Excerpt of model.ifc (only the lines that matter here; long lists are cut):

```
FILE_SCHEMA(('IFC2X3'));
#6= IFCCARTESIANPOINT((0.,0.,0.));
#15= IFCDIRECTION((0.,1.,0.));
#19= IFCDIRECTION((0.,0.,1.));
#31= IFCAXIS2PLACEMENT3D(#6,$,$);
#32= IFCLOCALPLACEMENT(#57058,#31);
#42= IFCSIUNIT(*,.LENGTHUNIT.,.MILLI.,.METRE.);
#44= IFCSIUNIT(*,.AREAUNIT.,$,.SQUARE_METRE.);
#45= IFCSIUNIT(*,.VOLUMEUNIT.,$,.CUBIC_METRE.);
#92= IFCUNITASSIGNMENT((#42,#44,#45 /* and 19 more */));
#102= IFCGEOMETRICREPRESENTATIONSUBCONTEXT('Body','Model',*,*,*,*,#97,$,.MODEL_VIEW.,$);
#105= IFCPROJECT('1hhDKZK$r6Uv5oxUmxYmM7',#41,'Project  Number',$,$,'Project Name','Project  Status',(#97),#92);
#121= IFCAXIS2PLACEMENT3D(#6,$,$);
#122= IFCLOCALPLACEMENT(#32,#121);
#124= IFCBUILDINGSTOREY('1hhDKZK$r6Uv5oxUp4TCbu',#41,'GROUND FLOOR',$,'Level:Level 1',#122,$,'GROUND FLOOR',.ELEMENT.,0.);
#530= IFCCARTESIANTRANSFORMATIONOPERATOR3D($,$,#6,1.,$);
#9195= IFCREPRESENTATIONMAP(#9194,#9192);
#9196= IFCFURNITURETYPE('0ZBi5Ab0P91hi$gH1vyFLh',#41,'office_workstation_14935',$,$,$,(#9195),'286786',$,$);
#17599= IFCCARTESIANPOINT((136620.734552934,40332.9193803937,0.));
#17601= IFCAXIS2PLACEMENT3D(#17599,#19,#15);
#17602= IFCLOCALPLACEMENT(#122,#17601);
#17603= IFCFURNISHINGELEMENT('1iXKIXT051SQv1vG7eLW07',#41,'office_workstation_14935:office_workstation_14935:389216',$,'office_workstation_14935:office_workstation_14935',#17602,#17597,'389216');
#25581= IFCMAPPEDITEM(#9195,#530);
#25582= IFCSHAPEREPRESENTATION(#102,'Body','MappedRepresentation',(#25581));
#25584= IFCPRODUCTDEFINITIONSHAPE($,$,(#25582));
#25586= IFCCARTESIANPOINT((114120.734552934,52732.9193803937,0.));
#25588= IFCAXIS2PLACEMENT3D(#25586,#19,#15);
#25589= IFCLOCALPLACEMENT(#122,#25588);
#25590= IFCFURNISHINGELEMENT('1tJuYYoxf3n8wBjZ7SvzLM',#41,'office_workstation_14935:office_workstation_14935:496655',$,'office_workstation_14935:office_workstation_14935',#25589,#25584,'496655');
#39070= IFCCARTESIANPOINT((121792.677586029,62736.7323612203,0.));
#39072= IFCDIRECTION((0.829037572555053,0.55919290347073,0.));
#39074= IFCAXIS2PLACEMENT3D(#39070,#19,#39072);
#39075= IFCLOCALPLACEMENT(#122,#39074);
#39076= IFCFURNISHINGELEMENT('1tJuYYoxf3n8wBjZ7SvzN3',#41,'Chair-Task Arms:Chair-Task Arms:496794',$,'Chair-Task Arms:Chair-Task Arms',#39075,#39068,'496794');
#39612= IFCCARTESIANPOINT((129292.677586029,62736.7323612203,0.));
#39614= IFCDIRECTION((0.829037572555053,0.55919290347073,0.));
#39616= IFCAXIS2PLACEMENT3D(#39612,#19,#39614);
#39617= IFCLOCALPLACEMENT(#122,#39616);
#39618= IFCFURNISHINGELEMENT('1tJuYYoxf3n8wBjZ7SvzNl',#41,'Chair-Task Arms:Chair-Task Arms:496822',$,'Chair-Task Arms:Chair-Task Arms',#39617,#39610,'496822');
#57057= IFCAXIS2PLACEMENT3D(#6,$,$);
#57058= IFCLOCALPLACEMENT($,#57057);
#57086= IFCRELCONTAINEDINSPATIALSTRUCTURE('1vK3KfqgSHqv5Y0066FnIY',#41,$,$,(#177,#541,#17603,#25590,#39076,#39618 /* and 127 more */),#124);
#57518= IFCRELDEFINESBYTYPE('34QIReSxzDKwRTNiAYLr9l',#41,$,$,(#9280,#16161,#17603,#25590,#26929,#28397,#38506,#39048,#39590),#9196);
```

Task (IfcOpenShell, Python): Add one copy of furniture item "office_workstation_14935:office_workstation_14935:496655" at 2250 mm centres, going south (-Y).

```python
import numpy as np
import ifcopenshell
import ifcopenshell.api.geometry
import ifcopenshell.api.root
import ifcopenshell.util.element
import ifcopenshell.util.placement
import ifcopenshell.util.unit

model = ifcopenshell.open("model.ifc")
unit_scale = ifcopenshell.util.unit.calculate_unit_scale(model)


def reuse_history(source, copy):
    """copy_class also copies each property set's owner history, people and application; keep the originals."""
    for rel in copy.IsDefinedBy:
        if rel.is_a("IfcRelDefinesByProperties") and (history := rel.RelatingPropertyDefinition.OwnerHistory):
            rel.RelatingPropertyDefinition.OwnerHistory = source.OwnerHistory
            ifcopenshell.util.element.remove_deep2(model, history)


source = model.by_guid("1tJuYYoxf3n8wBjZ7SvzLM")
base = ifcopenshell.util.placement.get_local_placement(source.ObjectPlacement)
step = np.array([0.0, -1.0, 0.0]) * 2.25 / unit_scale

for i in range(1, 2):
    copy = ifcopenshell.api.root.copy_class(model, product=source)
    copy.Representation = ifcopenshell.util.element.copy_deep(
        model, source.Representation, exclude=["IfcGeometricRepresentationContext", "IfcRepresentationMap"]
    )
    copy.Name = "office_workstation_14935:office_workstation_14935"
    copy.Tag = None
    reuse_history(source, copy)
    matrix = base.copy()
    matrix[:3, 3] += i * step
    print("added at", matrix[:3, 3].round(3) + 0.0)
    ifcopenshell.api.geometry.edit_object_placement(model, product=copy, matrix=matrix, is_si=False)

model.write("model_rev.ifc")
```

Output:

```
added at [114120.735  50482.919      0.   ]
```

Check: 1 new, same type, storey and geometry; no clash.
